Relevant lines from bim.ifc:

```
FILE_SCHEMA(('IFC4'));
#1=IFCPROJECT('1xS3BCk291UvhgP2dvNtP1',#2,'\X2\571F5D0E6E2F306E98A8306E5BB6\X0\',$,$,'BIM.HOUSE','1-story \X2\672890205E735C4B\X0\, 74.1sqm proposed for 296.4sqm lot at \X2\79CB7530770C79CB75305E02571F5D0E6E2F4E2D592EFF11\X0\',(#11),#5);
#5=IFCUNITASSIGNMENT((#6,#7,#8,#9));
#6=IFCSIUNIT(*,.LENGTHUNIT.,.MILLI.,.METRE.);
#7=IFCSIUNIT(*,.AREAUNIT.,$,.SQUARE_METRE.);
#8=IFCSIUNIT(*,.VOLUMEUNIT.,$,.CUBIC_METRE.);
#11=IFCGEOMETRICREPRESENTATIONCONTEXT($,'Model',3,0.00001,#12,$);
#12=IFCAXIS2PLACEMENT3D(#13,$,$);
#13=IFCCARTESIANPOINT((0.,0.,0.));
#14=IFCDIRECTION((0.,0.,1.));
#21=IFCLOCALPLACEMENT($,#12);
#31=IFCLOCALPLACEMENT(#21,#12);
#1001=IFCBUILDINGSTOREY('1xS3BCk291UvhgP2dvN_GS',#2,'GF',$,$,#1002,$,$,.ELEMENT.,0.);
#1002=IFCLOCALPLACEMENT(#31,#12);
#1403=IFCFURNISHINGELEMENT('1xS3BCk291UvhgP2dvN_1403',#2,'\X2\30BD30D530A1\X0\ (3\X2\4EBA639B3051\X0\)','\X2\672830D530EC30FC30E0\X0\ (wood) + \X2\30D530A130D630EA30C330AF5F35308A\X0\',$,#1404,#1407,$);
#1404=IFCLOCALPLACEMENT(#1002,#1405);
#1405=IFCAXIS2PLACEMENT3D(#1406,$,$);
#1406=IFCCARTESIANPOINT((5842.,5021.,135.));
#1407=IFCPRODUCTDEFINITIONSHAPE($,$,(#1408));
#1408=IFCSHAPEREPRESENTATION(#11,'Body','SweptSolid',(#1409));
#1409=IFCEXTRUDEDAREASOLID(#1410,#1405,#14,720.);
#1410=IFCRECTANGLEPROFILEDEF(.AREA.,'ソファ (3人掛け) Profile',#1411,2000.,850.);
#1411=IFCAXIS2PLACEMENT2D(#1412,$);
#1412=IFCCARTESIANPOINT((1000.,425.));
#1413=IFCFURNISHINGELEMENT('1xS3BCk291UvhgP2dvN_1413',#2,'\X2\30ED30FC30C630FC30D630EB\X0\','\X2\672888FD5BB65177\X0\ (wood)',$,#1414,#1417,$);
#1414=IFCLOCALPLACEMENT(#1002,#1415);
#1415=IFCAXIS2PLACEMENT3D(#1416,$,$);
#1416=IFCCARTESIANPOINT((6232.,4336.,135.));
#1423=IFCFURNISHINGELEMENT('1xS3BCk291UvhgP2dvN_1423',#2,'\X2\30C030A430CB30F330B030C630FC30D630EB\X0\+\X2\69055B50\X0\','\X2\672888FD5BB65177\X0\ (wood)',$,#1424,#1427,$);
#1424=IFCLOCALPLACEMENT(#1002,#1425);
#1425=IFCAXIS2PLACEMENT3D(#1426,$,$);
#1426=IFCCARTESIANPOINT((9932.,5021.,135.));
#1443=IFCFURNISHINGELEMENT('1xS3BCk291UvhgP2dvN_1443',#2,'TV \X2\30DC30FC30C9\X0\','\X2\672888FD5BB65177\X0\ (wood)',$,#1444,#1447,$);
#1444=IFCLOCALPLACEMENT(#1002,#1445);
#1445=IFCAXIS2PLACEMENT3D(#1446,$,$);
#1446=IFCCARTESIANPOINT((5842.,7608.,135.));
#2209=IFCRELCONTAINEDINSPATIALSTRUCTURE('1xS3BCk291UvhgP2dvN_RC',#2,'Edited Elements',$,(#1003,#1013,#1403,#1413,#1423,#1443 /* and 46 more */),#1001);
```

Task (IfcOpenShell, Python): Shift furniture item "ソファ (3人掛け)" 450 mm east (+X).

```python
import ifcopenshell
import ifcopenshell.api.geometry
import ifcopenshell.util.placement
import ifcopenshell.util.unit

model = ifcopenshell.open("bim.ifc")
unit_scale = ifcopenshell.util.unit.calculate_unit_scale(model)

item = model.by_id(1403)
matrix = ifcopenshell.util.placement.get_local_placement(item.ObjectPlacement)
matrix[0, 3] += 0.45 / unit_scale
ifcopenshell.api.geometry.edit_object_placement(model, product=item, matrix=matrix, is_si=False)

print(ifcopenshell.util.placement.get_local_placement(item.ObjectPlacement).round(3) + 0.0)

model.write("bim_v2.ifc")
```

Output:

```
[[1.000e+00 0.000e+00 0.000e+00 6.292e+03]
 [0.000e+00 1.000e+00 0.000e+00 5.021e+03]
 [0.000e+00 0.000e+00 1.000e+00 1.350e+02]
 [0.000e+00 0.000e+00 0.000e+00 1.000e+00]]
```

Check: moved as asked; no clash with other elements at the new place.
